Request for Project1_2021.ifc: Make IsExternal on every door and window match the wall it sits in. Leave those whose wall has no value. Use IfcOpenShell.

First a look at what the model holds.

```python
import ifcopenshell
import ifcopenshell.util.element

model = ifcopenshell.open("Project1_2021.ifc")
print(model.schema)
seen = {}
for e in model.by_type("IfcDoor") + model.by_type("IfcWindow"):
    if not e.FillsVoids:
        continue
    host = e.FillsVoids[0].RelatingOpeningElement.VoidsElements[0].RelatingBuildingElement
    own = ifcopenshell.util.element.get_pset(e, f"Pset_{e.is_a()[3:].removesuffix('StandardCase')}Common", "IsExternal")
    wall = ifcopenshell.util.element.get_pset(host, "Pset_WallCommon", "IsExternal")
    seen[e.is_a(), own, wall] = seen.get((e.is_a(), own, wall), 0) + 1
for (cls, own, wall), count in sorted(seen.items(), key=str):
    print(count, cls, "IsExternal:", own, "| host wall:", wall)
```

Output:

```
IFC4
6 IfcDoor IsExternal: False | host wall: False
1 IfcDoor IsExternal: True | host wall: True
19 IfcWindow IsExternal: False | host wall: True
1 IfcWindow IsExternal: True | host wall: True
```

```python
import ifcopenshell
import ifcopenshell.api.pset
import ifcopenshell.util.element

model = ifcopenshell.open("Project1_2021.ifc")

count = 0
for ifc_class, pset_name in (("IfcDoor", "Pset_DoorCommon"), ("IfcWindow", "Pset_WindowCommon")):
    for e in model.by_type(ifc_class):
        if not e.FillsVoids:
            continue
        host = e.FillsVoids[0].RelatingOpeningElement.VoidsElements[0].RelatingBuildingElement
        external = ifcopenshell.util.element.get_pset(host, "Pset_WallCommon", "IsExternal")
        if external is None or ifcopenshell.util.element.get_pset(e, pset_name, "IsExternal") == external:
            continue
        pset = ifcopenshell.api.pset.add_pset(model, product=e, name=pset_name)
        ifcopenshell.api.pset.edit_pset(model, pset=pset, properties={"IsExternal": external})
        count += 1

print(count, "updated")

model.write("Project1_2021_rev.ifc")
```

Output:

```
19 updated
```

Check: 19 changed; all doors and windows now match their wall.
